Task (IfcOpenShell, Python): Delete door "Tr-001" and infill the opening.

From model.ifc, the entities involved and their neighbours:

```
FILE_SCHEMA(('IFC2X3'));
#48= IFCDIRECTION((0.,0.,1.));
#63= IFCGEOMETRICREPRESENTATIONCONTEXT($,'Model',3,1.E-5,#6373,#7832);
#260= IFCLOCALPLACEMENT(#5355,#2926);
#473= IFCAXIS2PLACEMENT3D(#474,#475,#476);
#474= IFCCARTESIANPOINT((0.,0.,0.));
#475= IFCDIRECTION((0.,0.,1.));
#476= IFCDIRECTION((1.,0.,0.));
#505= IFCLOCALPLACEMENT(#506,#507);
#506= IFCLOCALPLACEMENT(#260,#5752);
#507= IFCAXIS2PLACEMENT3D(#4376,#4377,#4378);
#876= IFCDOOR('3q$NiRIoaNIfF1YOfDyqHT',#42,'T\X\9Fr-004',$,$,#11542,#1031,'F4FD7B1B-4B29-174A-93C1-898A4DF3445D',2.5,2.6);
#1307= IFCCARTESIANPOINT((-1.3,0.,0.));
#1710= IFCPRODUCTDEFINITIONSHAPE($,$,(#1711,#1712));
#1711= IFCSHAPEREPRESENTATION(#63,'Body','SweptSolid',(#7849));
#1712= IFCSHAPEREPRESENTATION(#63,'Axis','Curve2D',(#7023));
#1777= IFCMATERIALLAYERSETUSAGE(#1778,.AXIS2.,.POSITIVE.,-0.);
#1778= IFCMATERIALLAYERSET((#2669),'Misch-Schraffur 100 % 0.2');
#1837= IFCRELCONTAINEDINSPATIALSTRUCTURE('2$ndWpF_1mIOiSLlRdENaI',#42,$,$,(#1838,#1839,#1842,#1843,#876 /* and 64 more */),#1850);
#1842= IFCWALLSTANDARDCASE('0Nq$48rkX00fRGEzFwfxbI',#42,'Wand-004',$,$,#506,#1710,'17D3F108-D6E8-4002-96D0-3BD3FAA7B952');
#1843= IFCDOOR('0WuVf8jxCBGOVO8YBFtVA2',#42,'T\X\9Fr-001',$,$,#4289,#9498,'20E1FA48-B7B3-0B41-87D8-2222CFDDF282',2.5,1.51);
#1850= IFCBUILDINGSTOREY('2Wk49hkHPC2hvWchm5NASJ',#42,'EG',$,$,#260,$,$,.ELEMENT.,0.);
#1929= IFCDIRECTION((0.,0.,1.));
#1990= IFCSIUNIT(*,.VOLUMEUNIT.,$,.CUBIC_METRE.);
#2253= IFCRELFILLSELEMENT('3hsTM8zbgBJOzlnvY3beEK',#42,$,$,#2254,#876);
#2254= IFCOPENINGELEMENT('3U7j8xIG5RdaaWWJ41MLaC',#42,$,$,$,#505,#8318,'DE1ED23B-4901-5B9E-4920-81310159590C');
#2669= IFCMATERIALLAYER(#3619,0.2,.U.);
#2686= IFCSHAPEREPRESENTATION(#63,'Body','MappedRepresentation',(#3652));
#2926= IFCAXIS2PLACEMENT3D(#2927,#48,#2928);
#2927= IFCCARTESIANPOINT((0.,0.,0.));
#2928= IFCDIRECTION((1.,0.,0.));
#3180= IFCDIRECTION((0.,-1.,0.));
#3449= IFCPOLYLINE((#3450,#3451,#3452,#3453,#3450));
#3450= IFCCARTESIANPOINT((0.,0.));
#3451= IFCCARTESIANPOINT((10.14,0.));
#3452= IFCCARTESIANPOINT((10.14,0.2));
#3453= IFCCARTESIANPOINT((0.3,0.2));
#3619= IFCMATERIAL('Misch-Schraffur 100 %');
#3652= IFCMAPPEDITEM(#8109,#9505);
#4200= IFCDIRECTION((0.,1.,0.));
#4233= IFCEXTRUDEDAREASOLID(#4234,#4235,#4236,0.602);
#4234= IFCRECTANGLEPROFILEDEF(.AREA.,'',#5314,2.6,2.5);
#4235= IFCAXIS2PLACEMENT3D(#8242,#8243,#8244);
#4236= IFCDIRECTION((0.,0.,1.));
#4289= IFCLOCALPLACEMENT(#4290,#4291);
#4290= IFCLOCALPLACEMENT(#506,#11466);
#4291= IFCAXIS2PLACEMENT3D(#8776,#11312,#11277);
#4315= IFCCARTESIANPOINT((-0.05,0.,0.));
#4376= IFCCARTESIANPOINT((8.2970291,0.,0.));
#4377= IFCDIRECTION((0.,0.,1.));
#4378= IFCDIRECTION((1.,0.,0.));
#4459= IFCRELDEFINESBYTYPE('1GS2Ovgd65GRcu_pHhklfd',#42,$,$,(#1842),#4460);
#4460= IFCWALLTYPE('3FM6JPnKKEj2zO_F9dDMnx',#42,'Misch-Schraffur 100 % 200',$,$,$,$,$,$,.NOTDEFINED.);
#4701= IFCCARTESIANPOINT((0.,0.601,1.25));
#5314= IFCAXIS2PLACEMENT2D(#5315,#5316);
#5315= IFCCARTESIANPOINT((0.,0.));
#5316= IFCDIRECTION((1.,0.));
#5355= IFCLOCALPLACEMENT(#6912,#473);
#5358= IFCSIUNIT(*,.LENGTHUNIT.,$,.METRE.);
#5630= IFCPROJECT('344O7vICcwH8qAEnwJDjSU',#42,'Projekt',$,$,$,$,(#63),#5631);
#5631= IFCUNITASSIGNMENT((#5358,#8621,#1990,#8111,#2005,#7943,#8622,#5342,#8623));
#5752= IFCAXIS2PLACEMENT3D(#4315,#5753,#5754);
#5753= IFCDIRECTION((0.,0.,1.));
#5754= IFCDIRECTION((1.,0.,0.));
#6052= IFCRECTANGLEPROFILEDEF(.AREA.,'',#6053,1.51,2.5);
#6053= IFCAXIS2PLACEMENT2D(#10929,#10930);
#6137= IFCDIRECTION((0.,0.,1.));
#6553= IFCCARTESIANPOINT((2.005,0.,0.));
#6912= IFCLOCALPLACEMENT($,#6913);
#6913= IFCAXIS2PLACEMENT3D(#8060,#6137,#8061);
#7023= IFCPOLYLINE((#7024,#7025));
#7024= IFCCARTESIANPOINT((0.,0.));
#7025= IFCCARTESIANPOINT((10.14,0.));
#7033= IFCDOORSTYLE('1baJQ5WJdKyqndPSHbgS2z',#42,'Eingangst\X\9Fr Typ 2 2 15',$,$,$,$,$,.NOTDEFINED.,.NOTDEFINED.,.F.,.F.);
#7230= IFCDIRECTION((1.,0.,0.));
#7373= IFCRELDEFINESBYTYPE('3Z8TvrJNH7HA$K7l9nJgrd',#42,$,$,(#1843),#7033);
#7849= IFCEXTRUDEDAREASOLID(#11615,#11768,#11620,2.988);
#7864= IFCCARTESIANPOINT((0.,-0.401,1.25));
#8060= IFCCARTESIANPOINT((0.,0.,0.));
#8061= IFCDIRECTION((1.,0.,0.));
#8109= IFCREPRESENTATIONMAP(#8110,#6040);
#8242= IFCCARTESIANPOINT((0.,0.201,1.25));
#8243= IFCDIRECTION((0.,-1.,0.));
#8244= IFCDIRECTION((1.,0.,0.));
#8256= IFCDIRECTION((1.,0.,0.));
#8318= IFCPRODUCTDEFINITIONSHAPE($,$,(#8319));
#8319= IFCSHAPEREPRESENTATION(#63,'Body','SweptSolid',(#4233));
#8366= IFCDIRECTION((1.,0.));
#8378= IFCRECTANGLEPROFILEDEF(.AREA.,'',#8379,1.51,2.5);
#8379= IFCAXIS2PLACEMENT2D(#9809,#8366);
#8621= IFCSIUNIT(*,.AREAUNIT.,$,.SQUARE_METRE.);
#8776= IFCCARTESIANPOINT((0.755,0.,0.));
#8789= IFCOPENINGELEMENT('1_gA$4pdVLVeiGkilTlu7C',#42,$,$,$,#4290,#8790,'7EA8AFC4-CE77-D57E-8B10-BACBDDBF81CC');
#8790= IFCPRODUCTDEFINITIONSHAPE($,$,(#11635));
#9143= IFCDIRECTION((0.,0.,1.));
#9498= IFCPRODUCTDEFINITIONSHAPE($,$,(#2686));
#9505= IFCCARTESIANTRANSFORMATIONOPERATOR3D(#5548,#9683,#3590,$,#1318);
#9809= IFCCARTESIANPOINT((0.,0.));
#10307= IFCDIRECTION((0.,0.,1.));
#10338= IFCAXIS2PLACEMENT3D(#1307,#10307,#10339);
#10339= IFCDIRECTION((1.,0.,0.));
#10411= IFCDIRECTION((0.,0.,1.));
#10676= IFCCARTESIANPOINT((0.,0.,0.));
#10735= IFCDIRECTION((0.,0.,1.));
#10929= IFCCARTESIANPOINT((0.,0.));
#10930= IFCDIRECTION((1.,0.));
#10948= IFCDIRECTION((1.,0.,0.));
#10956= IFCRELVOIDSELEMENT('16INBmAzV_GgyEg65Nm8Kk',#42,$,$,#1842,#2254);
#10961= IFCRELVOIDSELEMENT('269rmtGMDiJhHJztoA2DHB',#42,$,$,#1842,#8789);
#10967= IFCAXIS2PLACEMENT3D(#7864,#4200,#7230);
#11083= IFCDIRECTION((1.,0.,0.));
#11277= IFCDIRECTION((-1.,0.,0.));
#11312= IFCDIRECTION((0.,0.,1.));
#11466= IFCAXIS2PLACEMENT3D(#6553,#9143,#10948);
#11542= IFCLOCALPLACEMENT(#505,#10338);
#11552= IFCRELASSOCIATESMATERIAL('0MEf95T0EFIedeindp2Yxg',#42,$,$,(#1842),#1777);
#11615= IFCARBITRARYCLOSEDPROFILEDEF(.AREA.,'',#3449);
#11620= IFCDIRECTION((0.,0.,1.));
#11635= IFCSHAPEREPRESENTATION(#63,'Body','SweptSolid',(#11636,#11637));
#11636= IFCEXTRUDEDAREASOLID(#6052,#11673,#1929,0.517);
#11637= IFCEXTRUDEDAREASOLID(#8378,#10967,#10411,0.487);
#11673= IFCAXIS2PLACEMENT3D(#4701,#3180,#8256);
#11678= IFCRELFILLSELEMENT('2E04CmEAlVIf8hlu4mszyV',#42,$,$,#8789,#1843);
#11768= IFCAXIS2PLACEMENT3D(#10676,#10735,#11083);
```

```python
import ifcopenshell
import ifcopenshell.api.feature
import ifcopenshell.api.root
import ifcopenshell.geom
import ifcopenshell.util.shape

model = ifcopenshell.open("model.ifc")
settings = ifcopenshell.geom.settings()


def volume(element):
    """Net volume in cubic metres, openings subtracted."""
    shape = ifcopenshell.geom.create_shape(settings, element)
    return ifcopenshell.util.shape.get_volume(shape.geometry)


door = model.by_guid("0WuVf8jxCBGOVO8YBFtVA2")
opening = door.FillsVoids[0].RelatingOpeningElement
wall = opening.VoidsElements[0].RelatingBuildingElement
before = volume(wall)

ifcopenshell.api.root.remove_product(model, product=door)
ifcopenshell.api.feature.remove_feature(model, feature=opening)

after = volume(wall)

print(f"wall volume {before:.3f} -> {after:.3f} m3")

model.write("model-out.ifc")
```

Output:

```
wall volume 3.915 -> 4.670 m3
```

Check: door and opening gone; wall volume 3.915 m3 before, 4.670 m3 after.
